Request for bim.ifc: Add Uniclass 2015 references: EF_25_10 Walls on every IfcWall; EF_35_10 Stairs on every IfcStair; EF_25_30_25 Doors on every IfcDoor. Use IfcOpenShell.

First a look at what the model holds.

```python
import ifcopenshell

model = ifcopenshell.open("bim.ifc")
print(model.schema)
print("classifications:", [c.Name for c in model.by_type("IfcClassification")])
for ifc_class in ("IfcDoor", "IfcRoof", "IfcStair", "IfcWall", "IfcWindow"):
    print(ifc_class, len(model.by_type(ifc_class)))
```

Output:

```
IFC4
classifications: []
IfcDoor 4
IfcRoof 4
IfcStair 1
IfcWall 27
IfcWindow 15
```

```python
import ifcopenshell
import ifcopenshell.api.classification

model = ifcopenshell.open("bim.ifc")

system = ifcopenshell.api.classification.add_classification(model, classification="Uniclass 2015")

codes = {
    "IfcWall": ("EF_25_10", "Walls"),
    "IfcStair": ("EF_35_10", "Stairs"),
    "IfcDoor": ("EF_25_30_25", "Doors"),
}
for ifc_class, (code, name) in codes.items():
    products = model.by_type(ifc_class)
    ifcopenshell.api.classification.add_reference(
        model, products=products, classification=system, identification=code, name=name
    )
    print(code, len(products))

model.write("bim_rev.ifc")
```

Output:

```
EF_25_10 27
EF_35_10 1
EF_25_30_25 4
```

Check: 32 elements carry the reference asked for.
